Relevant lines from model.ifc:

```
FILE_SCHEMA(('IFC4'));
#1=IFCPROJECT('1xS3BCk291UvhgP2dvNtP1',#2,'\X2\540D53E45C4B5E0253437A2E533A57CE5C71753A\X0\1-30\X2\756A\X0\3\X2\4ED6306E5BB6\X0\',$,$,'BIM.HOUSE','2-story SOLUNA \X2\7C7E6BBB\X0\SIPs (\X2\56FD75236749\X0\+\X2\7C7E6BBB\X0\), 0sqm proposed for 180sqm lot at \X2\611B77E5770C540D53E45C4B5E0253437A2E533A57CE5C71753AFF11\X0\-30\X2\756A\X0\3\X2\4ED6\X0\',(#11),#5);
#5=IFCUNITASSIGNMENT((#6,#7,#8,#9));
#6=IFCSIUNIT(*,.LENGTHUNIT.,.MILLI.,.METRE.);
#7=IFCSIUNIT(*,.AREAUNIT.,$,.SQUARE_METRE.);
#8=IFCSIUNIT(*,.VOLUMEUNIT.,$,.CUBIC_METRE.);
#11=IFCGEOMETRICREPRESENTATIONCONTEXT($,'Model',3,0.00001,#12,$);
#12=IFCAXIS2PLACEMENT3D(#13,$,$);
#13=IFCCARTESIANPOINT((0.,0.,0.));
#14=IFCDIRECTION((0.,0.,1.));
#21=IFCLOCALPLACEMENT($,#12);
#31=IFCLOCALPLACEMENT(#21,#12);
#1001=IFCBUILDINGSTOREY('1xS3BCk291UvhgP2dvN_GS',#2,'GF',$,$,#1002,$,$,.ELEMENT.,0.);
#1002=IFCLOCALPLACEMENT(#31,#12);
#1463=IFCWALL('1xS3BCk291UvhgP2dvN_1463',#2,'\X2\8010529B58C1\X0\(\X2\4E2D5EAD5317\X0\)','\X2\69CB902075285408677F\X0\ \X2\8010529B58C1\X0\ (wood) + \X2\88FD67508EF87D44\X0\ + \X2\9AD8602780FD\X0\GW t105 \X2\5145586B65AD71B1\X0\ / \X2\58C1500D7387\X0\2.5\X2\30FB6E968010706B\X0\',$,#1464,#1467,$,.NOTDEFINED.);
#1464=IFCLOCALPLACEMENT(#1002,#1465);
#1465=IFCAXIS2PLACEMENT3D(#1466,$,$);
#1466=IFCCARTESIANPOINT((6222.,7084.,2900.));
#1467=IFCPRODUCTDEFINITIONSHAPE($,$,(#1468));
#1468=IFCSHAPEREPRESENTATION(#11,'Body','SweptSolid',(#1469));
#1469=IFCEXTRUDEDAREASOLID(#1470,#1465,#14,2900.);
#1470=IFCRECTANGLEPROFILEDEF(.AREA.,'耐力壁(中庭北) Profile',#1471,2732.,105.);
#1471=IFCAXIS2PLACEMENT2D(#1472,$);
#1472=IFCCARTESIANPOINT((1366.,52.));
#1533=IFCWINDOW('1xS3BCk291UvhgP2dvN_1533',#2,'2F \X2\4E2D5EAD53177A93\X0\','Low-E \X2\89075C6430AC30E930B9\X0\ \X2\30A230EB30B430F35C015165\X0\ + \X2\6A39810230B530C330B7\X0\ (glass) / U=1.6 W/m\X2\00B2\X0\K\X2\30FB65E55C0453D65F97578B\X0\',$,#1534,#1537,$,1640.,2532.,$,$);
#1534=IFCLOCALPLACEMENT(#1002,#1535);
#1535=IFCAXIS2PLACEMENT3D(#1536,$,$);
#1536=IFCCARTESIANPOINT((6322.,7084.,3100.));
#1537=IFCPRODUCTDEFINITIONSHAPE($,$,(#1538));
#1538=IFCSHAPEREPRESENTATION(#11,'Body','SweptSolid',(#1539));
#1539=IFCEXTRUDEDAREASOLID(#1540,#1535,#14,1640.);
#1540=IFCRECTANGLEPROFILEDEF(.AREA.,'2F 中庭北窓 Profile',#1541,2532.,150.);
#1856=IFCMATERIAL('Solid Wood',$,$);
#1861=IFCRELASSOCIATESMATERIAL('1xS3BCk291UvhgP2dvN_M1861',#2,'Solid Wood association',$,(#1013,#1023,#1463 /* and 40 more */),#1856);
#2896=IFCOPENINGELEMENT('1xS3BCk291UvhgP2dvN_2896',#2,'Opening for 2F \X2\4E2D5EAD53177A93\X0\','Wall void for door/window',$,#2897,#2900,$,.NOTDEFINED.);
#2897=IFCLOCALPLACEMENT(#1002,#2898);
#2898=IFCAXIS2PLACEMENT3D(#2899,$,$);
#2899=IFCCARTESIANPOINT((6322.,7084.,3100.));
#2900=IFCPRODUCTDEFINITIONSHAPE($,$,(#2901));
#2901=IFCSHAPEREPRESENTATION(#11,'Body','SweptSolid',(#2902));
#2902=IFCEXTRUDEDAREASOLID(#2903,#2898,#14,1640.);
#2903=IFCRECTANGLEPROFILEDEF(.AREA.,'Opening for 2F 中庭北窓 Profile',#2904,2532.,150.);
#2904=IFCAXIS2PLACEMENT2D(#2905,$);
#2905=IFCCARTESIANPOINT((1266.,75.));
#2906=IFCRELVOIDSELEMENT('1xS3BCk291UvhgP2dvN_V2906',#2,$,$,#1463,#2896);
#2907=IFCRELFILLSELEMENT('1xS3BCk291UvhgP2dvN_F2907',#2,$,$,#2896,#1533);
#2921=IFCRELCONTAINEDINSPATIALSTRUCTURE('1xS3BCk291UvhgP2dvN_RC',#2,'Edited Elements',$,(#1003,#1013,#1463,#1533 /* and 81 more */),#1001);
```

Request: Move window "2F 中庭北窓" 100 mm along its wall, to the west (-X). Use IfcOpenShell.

```python
import ifcopenshell
import ifcopenshell.api.geometry
import ifcopenshell.util.placement

model = ifcopenshell.open("model.ifc")

window = model.by_guid("1xS3BCk291UvhgP2dvN_1533")
opening = window.FillsVoids[0].RelatingOpeningElement
wall = opening.VoidsElements[0].RelatingBuildingElement

wall_matrix = ifcopenshell.util.placement.get_local_placement(wall.ObjectPlacement)
shift = wall_matrix[:3, 0] * -100.0
before = ifcopenshell.util.placement.get_local_placement(window.ObjectPlacement)[:3, 3].copy()

# The window is not placed relative to its opening, so move both.
for product in (opening, window):
    matrix = ifcopenshell.util.placement.get_local_placement(product.ObjectPlacement)
    matrix[:3, 3] += shift
    ifcopenshell.api.geometry.edit_object_placement(model, product=product, matrix=matrix, is_si=False)

after = ifcopenshell.util.placement.get_local_placement(window.ObjectPlacement)[:3, 3]
print("window moved by", (after - before).round(3) + 0.0)

model.write("model_v2.ifc")
```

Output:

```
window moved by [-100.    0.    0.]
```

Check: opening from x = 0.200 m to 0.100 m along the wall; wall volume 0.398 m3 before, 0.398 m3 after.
